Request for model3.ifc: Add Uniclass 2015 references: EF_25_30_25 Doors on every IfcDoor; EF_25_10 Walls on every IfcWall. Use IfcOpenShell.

First a look at what the model holds.

```python
import ifcopenshell

model = ifcopenshell.open("model3.ifc")
print(model.schema)
print("classifications:", [c.Name for c in model.by_type("IfcClassification")])
for ifc_class in ("IfcDoor", "IfcRoof", "IfcStair", "IfcWall", "IfcWindow"):
    print(ifc_class, len(model.by_type(ifc_class)))
```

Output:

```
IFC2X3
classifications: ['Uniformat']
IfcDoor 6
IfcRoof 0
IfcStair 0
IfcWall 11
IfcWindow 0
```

```python
import ifcopenshell
import ifcopenshell.api.classification

model = ifcopenshell.open("model3.ifc")

# IFC2X3 requires Source and Edition and has no link from the project to the system.
system = model.create_entity("IfcClassification", Source="NBS", Edition="2015", Name="Uniclass 2015")

codes = {
    "IfcDoor": ("EF_25_30_25", "Doors"),
    "IfcWall": ("EF_25_10", "Walls"),
}
for ifc_class, (code, name) in codes.items():
    products = model.by_type(ifc_class)
    ifcopenshell.api.classification.add_reference(
        model, products=products, classification=system, identification=code, name=name
    )
    print(code, len(products))

model.write("model3-out.ifc")
```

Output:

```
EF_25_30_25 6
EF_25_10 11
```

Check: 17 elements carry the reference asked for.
